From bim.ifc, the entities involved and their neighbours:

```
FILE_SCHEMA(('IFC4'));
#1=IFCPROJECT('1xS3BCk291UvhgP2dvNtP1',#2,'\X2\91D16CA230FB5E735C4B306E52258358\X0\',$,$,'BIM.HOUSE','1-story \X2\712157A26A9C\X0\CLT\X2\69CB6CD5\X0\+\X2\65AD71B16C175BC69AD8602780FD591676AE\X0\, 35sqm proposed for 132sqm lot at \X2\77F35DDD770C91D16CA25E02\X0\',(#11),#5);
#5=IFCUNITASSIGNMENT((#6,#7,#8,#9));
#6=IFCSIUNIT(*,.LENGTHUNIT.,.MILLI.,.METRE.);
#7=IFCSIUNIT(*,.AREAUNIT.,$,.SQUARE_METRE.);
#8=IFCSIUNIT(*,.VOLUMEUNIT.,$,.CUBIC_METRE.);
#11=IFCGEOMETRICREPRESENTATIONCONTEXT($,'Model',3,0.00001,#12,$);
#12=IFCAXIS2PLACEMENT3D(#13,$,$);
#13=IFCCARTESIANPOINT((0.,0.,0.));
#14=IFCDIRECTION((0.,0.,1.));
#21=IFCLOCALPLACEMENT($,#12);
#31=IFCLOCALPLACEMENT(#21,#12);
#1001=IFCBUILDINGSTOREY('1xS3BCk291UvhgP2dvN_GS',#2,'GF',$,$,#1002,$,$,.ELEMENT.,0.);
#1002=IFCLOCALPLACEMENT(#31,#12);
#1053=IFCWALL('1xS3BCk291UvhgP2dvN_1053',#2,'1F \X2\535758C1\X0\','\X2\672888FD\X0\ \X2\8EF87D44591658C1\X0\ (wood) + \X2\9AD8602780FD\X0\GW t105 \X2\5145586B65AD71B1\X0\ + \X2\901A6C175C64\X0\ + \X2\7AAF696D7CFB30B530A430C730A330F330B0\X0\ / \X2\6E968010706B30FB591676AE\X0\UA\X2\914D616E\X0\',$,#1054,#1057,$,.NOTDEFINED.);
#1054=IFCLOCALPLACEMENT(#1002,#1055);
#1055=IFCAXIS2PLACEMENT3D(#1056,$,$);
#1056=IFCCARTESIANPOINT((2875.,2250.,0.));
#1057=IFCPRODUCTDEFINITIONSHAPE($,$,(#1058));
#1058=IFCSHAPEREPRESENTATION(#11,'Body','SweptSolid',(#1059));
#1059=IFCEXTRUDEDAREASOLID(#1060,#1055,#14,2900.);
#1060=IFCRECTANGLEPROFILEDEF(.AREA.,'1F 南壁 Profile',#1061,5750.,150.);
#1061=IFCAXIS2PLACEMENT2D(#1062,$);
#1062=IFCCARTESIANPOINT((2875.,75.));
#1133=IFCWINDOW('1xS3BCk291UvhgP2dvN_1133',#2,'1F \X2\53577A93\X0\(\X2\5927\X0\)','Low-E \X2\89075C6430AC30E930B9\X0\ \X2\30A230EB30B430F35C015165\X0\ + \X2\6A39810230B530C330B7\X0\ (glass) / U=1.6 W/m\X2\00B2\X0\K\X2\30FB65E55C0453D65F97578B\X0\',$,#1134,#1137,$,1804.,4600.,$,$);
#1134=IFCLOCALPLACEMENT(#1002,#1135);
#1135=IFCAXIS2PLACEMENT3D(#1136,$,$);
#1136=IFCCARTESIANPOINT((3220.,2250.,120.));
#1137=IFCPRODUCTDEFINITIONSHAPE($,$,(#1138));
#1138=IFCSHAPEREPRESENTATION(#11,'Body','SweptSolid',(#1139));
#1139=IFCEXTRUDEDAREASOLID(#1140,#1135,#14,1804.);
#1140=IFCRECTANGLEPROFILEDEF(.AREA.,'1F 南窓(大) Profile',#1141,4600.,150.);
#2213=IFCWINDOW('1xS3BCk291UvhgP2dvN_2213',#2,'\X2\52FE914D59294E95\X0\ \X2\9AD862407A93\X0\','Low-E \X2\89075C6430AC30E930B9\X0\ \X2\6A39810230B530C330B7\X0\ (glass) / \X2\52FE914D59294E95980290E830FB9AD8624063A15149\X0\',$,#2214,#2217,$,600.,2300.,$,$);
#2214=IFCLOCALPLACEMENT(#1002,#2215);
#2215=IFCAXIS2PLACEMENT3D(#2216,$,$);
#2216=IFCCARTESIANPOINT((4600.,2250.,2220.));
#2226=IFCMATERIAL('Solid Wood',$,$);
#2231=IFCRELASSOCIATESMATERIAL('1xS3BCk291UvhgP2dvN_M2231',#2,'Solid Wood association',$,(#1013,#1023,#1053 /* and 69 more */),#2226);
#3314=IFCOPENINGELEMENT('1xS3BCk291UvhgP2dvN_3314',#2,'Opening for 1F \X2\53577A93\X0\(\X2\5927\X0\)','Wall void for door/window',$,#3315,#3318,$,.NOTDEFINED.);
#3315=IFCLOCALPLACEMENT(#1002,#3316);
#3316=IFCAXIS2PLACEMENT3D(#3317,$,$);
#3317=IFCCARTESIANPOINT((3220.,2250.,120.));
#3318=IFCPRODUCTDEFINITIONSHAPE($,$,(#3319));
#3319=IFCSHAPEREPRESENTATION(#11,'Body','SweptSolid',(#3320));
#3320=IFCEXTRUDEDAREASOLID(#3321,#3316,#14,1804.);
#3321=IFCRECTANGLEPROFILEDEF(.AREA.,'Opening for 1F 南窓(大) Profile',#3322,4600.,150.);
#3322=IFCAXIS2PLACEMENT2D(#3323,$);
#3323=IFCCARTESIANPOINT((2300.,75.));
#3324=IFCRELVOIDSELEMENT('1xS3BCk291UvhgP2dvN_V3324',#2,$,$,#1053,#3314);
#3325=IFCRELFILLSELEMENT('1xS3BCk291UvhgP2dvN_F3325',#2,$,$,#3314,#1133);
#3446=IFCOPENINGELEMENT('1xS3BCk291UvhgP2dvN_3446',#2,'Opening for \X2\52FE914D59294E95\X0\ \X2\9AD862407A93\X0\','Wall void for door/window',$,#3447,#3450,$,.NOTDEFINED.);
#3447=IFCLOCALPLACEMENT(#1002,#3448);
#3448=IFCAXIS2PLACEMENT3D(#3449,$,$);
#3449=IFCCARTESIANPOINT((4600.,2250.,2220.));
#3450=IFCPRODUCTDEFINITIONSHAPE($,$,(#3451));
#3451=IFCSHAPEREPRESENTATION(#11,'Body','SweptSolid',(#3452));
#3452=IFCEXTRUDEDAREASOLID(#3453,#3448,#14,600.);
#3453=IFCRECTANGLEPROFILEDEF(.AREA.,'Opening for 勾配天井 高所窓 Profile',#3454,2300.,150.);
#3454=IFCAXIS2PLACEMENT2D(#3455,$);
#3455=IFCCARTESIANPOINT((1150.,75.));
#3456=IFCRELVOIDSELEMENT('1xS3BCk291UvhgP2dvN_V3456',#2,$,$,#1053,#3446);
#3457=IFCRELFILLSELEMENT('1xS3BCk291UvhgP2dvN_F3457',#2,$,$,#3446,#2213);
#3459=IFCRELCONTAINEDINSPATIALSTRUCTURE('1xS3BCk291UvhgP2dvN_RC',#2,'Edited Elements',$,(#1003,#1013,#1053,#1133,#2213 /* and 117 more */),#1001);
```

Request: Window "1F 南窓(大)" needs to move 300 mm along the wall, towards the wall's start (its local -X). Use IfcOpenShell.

```python
import ifcopenshell
import ifcopenshell.api.geometry
import ifcopenshell.util.placement
import ifcopenshell.util.unit

model = ifcopenshell.open("bim.ifc")
unit_scale = ifcopenshell.util.unit.calculate_unit_scale(model)

window = model.by_guid("1xS3BCk291UvhgP2dvN_1133")
opening = window.FillsVoids[0].RelatingOpeningElement
wall = opening.VoidsElements[0].RelatingBuildingElement

wall_matrix = ifcopenshell.util.placement.get_local_placement(wall.ObjectPlacement)
shift = wall_matrix[:3, 0] * -0.3 / unit_scale
before = ifcopenshell.util.placement.get_local_placement(window.ObjectPlacement)[:3, 3].copy()

# The window is not placed relative to its opening, so move both.
for product in (opening, window):
    matrix = ifcopenshell.util.placement.get_local_placement(product.ObjectPlacement)
    matrix[:3, 3] += shift
    ifcopenshell.api.geometry.edit_object_placement(model, product=product, matrix=matrix, is_si=False)

after = ifcopenshell.util.placement.get_local_placement(window.ObjectPlacement)[:3, 3]
print("window moved by", (after - before).round(3) + 0.0)

model.write("bim_updated.ifc")
```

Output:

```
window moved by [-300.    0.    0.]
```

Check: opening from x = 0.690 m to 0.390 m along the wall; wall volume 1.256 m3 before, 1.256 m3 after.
